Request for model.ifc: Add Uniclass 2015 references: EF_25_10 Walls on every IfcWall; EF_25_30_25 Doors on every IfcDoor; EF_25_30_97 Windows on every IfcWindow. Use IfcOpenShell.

First a look at what the model holds.

```python
import ifcopenshell

model = ifcopenshell.open("model.ifc")
print(model.schema)
print("classifications:", [c.Name for c in model.by_type("IfcClassification")])
for ifc_class in ("IfcDoor", "IfcRoof", "IfcStair", "IfcWall", "IfcWindow"):
    print(ifc_class, len(model.by_type(ifc_class)))
```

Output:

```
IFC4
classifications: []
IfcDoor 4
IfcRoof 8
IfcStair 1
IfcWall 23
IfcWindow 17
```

```python
import ifcopenshell
import ifcopenshell.api.classification

model = ifcopenshell.open("model.ifc")

system = ifcopenshell.api.classification.add_classification(model, classification="Uniclass 2015")

codes = {
    "IfcWall": ("EF_25_10", "Walls"),
    "IfcDoor": ("EF_25_30_25", "Doors"),
    "IfcWindow": ("EF_25_30_97", "Windows"),
}
for ifc_class, (code, name) in codes.items():
    products = model.by_type(ifc_class)
    ifcopenshell.api.classification.add_reference(
        model, products=products, classification=system, identification=code, name=name
    )
    print(code, len(products))

model.write("model_edited.ifc")
```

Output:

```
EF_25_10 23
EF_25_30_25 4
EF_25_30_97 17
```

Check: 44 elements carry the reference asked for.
